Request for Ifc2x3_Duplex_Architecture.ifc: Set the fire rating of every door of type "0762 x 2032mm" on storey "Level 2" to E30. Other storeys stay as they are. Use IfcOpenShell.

First a look at what the model holds.

```python
import ifcopenshell
import ifcopenshell.util.element

model = ifcopenshell.open("Ifc2x3_Duplex_Architecture.ifc")
print(model.schema)
storey = next(s for s in model.by_type("IfcBuildingStorey") if s.Name == "Level 2")
doors = [e for e in ifcopenshell.util.element.get_decomposition(storey) if e.is_a("IfcDoor")]
seen = {}
for e in doors:
    element_type = ifcopenshell.util.element.get_type(e)
    key = (element_type.Name if element_type != e and element_type else None, ifcopenshell.util.element.get_pset(e, "Pset_DoorCommon", "FireRating"))
    seen[key] = seen.get(key, 0) + 1
for (name, value), count in sorted(seen.items(), key=str):
    print(count, "x", name, "|", value)
```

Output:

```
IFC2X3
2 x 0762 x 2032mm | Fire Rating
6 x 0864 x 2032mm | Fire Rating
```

```python
import ifcopenshell
import ifcopenshell.api.pset
import ifcopenshell.util.element

model = ifcopenshell.open("Ifc2x3_Duplex_Architecture.ifc")

storey = next(s for s in model.by_type("IfcBuildingStorey") if s.Name == "Level 2")
doors = [e for e in ifcopenshell.util.element.get_decomposition(storey) if e.is_a("IfcDoor")]

count = 0
for e in doors:
    element_type = ifcopenshell.util.element.get_type(e)
    if element_type in (None, e) or element_type.Name != "0762 x 2032mm":
        continue
    # add_pset returns the element's existing set when there is one.
    pset = ifcopenshell.api.pset.add_pset(model, product=e, name="Pset_DoorCommon")
    ifcopenshell.api.pset.edit_pset(model, pset=pset, properties={"FireRating": "E30"})
    count += 1

print(count, "doors updated")

model.write("Ifc2x3_Duplex_Architecture_edited.ifc")
```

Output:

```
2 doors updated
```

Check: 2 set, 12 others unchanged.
